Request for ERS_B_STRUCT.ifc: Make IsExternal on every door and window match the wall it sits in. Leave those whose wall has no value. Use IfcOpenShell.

First a look at what the model holds.

```python
import ifcopenshell
import ifcopenshell.util.element

model = ifcopenshell.open("ERS_B_STRUCT.ifc")
print(model.schema)
seen = {}
for e in model.by_type("IfcDoor") + model.by_type("IfcWindow"):
    if not e.FillsVoids:
        continue
    host = e.FillsVoids[0].RelatingOpeningElement.VoidsElements[0].RelatingBuildingElement
    own = ifcopenshell.util.element.get_pset(e, f"Pset_{e.is_a()[3:].removesuffix('StandardCase')}Common", "IsExternal")
    wall = ifcopenshell.util.element.get_pset(host, "Pset_WallCommon", "IsExternal")
    seen[e.is_a(), own, wall] = seen.get((e.is_a(), own, wall), 0) + 1
for (cls, own, wall), count in sorted(seen.items(), key=str):
    print(count, cls, "IsExternal:", own, "| host wall:", wall)
```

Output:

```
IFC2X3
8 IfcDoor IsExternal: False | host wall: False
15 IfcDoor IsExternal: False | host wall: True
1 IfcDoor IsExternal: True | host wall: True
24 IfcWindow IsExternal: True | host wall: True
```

```python
import ifcopenshell
import ifcopenshell.api.pset
import ifcopenshell.util.element

model = ifcopenshell.open("ERS_B_STRUCT.ifc")

count = 0
for ifc_class, pset_name in (("IfcDoor", "Pset_DoorCommon"), ("IfcWindow", "Pset_WindowCommon")):
    for e in model.by_type(ifc_class):
        if not e.FillsVoids:
            continue
        host = e.FillsVoids[0].RelatingOpeningElement.VoidsElements[0].RelatingBuildingElement
        external = ifcopenshell.util.element.get_pset(host, "Pset_WallCommon", "IsExternal")
        if external is None or ifcopenshell.util.element.get_pset(e, pset_name, "IsExternal") == external:
            continue
        pset = ifcopenshell.api.pset.add_pset(model, product=e, name=pset_name)
        ifcopenshell.api.pset.edit_pset(model, pset=pset, properties={"IsExternal": external})
        count += 1

print(count, "updated")

model.write("ERS_B_STRUCT_rev.ifc")
```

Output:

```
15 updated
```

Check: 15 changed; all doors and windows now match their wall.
